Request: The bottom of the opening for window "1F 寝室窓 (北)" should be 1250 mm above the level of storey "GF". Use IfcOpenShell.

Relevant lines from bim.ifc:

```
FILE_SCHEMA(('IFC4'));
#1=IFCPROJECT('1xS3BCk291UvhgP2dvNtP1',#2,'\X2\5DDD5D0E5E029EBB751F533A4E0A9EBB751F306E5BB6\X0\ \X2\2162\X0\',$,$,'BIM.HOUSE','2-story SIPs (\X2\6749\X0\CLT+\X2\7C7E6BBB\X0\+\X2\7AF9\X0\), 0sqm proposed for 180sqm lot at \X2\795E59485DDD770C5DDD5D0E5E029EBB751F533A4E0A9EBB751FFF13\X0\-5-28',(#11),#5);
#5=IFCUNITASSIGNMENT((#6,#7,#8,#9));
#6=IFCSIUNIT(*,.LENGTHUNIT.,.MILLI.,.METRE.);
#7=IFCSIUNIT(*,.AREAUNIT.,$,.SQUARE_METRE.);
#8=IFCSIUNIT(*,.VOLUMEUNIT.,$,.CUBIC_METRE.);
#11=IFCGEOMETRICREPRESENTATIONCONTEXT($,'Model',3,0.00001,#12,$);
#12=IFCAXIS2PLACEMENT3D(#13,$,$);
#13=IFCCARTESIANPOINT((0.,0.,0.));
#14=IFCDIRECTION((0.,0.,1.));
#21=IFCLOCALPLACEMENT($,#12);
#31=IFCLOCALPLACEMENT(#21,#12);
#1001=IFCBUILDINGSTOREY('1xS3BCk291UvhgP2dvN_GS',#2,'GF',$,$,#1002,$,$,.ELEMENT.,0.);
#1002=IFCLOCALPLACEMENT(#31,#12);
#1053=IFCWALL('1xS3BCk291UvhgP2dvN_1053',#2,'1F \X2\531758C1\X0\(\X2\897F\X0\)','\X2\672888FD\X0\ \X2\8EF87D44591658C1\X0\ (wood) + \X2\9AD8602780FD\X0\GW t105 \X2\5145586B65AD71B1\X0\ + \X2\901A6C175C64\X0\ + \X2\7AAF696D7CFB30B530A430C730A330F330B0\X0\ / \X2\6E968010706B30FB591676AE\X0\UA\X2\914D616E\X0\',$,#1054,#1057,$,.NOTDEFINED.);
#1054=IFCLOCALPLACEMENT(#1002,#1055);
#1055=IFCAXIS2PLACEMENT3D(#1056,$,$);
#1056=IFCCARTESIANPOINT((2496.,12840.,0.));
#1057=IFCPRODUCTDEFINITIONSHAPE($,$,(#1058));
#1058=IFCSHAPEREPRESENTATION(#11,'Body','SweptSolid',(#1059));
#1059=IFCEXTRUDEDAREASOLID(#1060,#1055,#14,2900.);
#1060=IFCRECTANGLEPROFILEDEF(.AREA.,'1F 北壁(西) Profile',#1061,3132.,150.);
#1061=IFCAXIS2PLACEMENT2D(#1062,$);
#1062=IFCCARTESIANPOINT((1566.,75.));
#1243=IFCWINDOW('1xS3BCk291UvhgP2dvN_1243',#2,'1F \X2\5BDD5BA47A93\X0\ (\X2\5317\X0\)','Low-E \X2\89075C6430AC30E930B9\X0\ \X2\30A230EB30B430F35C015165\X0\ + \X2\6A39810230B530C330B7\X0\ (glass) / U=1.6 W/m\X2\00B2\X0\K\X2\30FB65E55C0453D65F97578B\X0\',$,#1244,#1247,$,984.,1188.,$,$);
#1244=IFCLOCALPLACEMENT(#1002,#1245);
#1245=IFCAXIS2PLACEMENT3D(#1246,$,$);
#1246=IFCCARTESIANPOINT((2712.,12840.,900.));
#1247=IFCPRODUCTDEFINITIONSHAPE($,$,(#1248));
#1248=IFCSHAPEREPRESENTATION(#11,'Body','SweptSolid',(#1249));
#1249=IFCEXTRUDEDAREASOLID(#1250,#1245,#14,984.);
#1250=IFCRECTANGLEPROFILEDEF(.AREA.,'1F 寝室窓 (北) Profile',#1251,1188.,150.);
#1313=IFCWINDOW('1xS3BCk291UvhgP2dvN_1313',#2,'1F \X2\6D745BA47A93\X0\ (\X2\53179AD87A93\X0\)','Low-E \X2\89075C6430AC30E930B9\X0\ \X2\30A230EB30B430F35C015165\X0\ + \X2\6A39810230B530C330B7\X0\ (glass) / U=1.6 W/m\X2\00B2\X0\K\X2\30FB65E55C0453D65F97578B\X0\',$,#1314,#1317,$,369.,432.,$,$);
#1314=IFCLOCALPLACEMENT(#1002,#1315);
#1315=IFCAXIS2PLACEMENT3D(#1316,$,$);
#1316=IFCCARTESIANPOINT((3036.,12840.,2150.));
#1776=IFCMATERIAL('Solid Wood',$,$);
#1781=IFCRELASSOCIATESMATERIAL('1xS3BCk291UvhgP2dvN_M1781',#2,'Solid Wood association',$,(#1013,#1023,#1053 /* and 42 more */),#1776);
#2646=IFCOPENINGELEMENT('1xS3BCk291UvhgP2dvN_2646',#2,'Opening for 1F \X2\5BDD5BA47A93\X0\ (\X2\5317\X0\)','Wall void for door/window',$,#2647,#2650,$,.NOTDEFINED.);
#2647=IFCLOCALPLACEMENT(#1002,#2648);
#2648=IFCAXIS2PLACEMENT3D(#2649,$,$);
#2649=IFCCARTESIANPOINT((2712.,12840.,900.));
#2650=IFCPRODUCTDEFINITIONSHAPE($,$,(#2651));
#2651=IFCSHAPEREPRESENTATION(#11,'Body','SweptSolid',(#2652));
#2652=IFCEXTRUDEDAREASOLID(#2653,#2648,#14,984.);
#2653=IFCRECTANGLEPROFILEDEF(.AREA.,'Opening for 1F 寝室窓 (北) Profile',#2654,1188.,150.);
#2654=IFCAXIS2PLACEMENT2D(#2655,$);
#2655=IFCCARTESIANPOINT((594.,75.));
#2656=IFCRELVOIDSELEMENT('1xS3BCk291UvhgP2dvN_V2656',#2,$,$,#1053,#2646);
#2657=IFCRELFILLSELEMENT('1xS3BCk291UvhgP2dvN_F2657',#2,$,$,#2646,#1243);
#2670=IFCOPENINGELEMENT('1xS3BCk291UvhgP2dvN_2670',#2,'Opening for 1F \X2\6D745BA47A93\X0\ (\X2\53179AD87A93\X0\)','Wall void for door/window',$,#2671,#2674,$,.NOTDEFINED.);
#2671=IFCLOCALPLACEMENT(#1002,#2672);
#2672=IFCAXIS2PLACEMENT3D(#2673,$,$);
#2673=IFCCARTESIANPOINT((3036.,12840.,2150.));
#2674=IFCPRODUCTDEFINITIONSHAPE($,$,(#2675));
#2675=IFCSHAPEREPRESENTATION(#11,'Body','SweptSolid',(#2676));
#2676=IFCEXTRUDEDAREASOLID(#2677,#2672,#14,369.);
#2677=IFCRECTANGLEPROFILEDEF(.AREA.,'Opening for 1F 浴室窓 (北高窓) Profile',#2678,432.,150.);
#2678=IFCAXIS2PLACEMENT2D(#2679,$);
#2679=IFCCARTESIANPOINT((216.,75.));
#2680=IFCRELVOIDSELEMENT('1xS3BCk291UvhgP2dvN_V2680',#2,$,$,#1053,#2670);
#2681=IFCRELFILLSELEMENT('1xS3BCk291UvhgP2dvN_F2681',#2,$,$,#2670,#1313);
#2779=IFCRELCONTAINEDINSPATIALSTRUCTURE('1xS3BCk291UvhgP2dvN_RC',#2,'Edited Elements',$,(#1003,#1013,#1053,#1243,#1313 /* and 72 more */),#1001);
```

```python
import numpy as np
import ifcopenshell
import ifcopenshell.api.geometry
import ifcopenshell.geom
import ifcopenshell.util.element
import ifcopenshell.util.placement
import ifcopenshell.util.shape
import ifcopenshell.util.unit

model = ifcopenshell.open("bim.ifc")
unit_scale = ifcopenshell.util.unit.calculate_unit_scale(model)

window = model.by_guid("1xS3BCk291UvhgP2dvN_1243")
opening = window.FillsVoids[0].RelatingOpeningElement
storey = ifcopenshell.util.element.get_container(window, ifc_class="IfcBuildingStorey")
level = ifcopenshell.util.placement.get_local_placement(storey.ObjectPlacement)[2, 3]

# The opening's origin need not be at the sill, so measure its lowest point.
shape = ifcopenshell.geom.create_shape(ifcopenshell.geom.settings(), opening)
bottom = ifcopenshell.util.shape.get_shape_bottom_elevation(shape, shape.geometry) / unit_scale
dz = level + 1.25 / unit_scale - bottom

shift = np.array([0.0, 0.0, dz])
# The window is not placed relative to its opening, so move both.
for product in (opening, window):
    matrix = ifcopenshell.util.placement.get_local_placement(product.ObjectPlacement)
    matrix[:3, 3] += shift
    ifcopenshell.api.geometry.edit_object_placement(model, product=product, matrix=matrix, is_si=False)

print(f"moved by {dz * unit_scale:+.3f} m")

model.write("bim_updated.ifc")
```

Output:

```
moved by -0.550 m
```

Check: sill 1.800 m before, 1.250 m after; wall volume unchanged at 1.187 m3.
